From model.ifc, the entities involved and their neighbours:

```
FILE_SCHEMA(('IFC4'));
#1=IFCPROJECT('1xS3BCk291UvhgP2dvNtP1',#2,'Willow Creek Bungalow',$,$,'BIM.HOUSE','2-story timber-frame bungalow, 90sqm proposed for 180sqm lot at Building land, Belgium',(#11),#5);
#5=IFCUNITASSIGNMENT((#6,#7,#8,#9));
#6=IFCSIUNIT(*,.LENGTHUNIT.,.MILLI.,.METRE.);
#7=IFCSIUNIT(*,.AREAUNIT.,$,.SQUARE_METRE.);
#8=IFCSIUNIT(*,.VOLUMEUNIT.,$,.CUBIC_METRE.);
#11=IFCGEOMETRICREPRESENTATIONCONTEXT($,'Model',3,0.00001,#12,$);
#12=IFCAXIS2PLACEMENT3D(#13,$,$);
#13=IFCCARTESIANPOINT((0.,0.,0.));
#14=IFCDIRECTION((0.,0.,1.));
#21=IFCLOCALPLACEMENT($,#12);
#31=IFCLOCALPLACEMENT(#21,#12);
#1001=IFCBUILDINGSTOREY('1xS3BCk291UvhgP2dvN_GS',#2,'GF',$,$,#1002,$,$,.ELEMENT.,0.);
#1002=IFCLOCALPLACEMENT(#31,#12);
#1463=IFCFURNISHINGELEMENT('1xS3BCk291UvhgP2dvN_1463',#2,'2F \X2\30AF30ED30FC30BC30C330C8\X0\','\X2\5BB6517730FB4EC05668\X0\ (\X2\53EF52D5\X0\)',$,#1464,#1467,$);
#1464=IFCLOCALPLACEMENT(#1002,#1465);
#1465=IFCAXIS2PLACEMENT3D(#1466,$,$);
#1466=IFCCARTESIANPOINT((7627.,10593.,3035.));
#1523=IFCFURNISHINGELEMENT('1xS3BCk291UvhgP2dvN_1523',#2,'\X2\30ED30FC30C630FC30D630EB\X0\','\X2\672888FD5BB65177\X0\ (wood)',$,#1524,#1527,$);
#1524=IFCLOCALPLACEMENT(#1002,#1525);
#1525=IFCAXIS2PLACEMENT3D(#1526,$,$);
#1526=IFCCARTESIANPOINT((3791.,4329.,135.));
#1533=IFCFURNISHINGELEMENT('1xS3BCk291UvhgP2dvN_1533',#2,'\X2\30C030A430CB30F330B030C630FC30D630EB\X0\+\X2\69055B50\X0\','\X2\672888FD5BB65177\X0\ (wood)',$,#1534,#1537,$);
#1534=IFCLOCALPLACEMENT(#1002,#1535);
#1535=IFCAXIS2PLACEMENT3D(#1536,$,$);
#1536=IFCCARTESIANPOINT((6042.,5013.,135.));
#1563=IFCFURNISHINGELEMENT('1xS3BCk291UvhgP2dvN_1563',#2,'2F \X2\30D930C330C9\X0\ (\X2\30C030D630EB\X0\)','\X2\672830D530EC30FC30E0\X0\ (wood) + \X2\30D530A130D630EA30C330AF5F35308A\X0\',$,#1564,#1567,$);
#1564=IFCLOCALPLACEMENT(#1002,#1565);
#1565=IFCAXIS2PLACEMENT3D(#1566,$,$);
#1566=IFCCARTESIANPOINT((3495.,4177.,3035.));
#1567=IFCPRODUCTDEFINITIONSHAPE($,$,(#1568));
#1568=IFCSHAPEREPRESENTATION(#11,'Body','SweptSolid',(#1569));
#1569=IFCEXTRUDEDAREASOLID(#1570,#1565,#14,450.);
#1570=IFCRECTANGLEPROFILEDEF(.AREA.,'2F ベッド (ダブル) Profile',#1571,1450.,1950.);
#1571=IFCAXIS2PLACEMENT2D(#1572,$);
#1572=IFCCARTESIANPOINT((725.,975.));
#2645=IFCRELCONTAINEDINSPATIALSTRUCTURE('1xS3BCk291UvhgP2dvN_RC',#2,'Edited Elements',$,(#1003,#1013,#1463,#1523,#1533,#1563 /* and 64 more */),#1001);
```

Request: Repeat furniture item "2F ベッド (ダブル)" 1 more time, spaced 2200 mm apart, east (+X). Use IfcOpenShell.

```python
import numpy as np
import ifcopenshell
import ifcopenshell.api.geometry
import ifcopenshell.api.root
import ifcopenshell.util.element
import ifcopenshell.util.placement
import ifcopenshell.util.unit

model = ifcopenshell.open("model.ifc")
unit_scale = ifcopenshell.util.unit.calculate_unit_scale(model)


def reuse_history(source, copy):
    """copy_class also copies each property set's owner history, people and application; keep the originals."""
    for rel in copy.IsDefinedBy:
        if rel.is_a("IfcRelDefinesByProperties") and (history := rel.RelatingPropertyDefinition.OwnerHistory):
            rel.RelatingPropertyDefinition.OwnerHistory = source.OwnerHistory
            ifcopenshell.util.element.remove_deep2(model, history)


source = model.by_id(1563)
base = ifcopenshell.util.placement.get_local_placement(source.ObjectPlacement)
step = np.array([1.0, 0.0, 0.0]) * 2.2 / unit_scale

for i in range(1, 2):
    copy = ifcopenshell.api.root.copy_class(model, product=source)
    copy.Representation = ifcopenshell.util.element.copy_deep(
        model, source.Representation, exclude=["IfcGeometricRepresentationContext", "IfcRepresentationMap"]
    )
    reuse_history(source, copy)
    matrix = base.copy()
    matrix[:3, 3] += i * step
    print("added at", matrix[:3, 3].round(3) + 0.0)
    ifcopenshell.api.geometry.edit_object_placement(model, product=copy, matrix=matrix, is_si=False)

model.write("model_rev.ifc")
```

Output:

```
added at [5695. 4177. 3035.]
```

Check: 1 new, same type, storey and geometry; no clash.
